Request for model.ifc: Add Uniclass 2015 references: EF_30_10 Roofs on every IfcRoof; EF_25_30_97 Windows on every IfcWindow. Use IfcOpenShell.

First a look at what the model holds.

```python
import ifcopenshell

model = ifcopenshell.open("model.ifc")
print(model.schema)
print("classifications:", [c.Name for c in model.by_type("IfcClassification")])
for ifc_class in ("IfcDoor", "IfcRoof", "IfcStair", "IfcWall", "IfcWindow"):
    print(ifc_class, len(model.by_type(ifc_class)))
```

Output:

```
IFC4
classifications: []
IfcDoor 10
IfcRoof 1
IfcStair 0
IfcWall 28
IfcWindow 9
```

```python
import ifcopenshell
import ifcopenshell.api.classification

model = ifcopenshell.open("model.ifc")

system = ifcopenshell.api.classification.add_classification(model, classification="Uniclass 2015")

codes = {
    "IfcRoof": ("EF_30_10", "Roofs"),
    "IfcWindow": ("EF_25_30_97", "Windows"),
}
for ifc_class, (code, name) in codes.items():
    products = model.by_type(ifc_class)
    ifcopenshell.api.classification.add_reference(
        model, products=products, classification=system, identification=code, name=name
    )
    print(code, len(products))

model.write("model_edited.ifc")
```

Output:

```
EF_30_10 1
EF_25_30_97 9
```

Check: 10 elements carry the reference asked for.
